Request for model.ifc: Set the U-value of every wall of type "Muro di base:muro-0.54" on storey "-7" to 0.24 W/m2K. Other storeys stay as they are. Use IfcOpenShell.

First a look at what the model holds.

```python
import ifcopenshell
import ifcopenshell.util.element

model = ifcopenshell.open("model.ifc")
print(model.schema)
storey = next(s for s in model.by_type("IfcBuildingStorey") if s.Name == "-7")
walls = [e for e in ifcopenshell.util.element.get_decomposition(storey) if e.is_a("IfcWall")]
seen = {}
for e in walls:
    element_type = ifcopenshell.util.element.get_type(e)
    key = (element_type.Name if element_type != e and element_type else None, ifcopenshell.util.element.get_pset(e, "Pset_WallCommon", "ThermalTransmittance"))
    seen[key] = seen.get(key, 0) + 1
for (name, value), count in sorted(seen.items(), key=str):
    print(count, "x", name, "|", value)
```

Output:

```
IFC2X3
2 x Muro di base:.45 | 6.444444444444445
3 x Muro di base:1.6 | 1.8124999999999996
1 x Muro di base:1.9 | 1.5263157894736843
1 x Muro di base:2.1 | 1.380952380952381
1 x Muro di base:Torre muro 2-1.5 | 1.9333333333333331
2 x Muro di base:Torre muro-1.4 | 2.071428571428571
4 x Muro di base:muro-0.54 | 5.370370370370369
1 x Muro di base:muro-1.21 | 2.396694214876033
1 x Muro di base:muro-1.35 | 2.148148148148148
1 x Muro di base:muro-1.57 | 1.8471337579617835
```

```python
import ifcopenshell
import ifcopenshell.api.pset
import ifcopenshell.util.element

model = ifcopenshell.open("model.ifc")

storey = next(s for s in model.by_type("IfcBuildingStorey") if s.Name == "-7")
walls = [e for e in ifcopenshell.util.element.get_decomposition(storey) if e.is_a("IfcWall")]

count = 0
for e in walls:
    element_type = ifcopenshell.util.element.get_type(e)
    if element_type in (None, e) or element_type.Name != "Muro di base:muro-0.54":
        continue
    # add_pset returns the element's existing set when there is one.
    pset = ifcopenshell.api.pset.add_pset(model, product=e, name="Pset_WallCommon")
    ifcopenshell.api.pset.edit_pset(model, pset=pset, properties={"ThermalTransmittance": 0.24})
    count += 1

print(count, "walls updated")

model.write("model_rev.ifc")
```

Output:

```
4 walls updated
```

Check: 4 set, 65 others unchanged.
